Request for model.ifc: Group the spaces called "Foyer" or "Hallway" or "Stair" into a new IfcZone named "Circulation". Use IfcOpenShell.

First a look at what the model holds.

```python
import ifcopenshell

model = ifcopenshell.open("model.ifc")
print(model.schema)
seen = {}
for space in model.by_type("IfcSpace"):
    seen[space.LongName] = seen.get(space.LongName, 0) + 1
for name, count in sorted(seen.items(), key=str):
    print(count, "x", name)
print("zones:", [z.Name for z in model.by_type("IfcZone")][:20])
```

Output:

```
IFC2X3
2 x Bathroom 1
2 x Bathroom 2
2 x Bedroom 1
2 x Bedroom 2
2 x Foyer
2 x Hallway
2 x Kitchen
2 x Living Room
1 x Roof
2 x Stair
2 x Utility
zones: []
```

```python
import ifcopenshell
import ifcopenshell.api.group
import ifcopenshell.api.root

model = ifcopenshell.open("model.ifc")

names = {"Foyer", "Hallway", "Stair"}
spaces = [s for s in model.by_type("IfcSpace") if s.LongName in names]

zone = ifcopenshell.api.root.create_entity(model, ifc_class="IfcZone", name="Circulation")
ifcopenshell.api.group.assign_group(model, products=spaces, group=zone)
print(len(spaces), "spaces in", zone.Name)

model.write("model_updated.ifc")
```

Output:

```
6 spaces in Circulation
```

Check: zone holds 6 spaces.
